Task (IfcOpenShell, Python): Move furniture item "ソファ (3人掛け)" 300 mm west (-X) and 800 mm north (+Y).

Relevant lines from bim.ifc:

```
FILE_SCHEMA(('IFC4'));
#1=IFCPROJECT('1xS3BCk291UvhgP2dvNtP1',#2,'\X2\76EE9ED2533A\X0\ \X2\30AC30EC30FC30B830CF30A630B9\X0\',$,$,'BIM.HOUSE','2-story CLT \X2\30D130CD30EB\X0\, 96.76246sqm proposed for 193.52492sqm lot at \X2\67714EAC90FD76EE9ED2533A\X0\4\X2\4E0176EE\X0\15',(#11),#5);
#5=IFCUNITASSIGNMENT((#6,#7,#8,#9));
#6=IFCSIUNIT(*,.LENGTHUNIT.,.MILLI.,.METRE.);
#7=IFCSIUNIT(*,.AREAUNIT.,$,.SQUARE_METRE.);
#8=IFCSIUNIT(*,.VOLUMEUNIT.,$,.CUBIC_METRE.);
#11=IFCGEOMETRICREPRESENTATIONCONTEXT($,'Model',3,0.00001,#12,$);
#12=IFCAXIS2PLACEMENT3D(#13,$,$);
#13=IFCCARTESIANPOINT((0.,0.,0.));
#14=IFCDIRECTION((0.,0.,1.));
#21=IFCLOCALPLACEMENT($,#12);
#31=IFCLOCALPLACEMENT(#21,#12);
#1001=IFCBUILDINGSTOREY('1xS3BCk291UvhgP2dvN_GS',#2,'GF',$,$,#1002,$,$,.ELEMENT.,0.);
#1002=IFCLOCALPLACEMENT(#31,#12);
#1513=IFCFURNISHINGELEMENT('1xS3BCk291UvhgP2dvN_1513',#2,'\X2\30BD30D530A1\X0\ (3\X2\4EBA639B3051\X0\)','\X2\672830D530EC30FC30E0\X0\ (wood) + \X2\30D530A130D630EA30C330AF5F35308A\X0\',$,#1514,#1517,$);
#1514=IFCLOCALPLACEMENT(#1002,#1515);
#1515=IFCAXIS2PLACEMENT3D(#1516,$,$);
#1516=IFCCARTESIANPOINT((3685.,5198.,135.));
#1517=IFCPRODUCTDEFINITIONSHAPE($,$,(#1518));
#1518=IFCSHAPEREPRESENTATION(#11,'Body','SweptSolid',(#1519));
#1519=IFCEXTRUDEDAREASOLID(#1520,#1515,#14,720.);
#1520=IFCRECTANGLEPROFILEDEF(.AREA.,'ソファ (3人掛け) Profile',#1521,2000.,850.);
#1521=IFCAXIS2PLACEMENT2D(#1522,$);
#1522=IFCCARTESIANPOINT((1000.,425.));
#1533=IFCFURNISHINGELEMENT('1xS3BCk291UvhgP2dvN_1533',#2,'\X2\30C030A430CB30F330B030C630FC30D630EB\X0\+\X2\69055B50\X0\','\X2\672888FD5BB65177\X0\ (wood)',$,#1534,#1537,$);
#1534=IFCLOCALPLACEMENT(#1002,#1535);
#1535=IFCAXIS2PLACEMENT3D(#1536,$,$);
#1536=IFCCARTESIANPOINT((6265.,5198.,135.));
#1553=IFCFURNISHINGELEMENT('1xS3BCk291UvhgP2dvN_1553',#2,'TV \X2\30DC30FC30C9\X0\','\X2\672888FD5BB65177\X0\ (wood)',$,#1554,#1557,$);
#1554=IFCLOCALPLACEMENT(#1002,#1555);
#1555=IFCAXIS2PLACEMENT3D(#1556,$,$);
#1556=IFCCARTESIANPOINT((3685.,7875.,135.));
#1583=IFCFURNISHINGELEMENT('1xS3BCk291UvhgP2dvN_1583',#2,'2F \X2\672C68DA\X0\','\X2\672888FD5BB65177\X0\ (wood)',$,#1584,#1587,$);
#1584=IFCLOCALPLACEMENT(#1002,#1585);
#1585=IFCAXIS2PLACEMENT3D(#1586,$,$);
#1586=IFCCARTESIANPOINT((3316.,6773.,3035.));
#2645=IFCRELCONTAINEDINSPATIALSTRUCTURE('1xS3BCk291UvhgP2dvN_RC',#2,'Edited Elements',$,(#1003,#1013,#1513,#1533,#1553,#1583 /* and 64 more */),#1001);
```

```python
import ifcopenshell
import ifcopenshell.api.geometry
import ifcopenshell.util.placement

model = ifcopenshell.open("bim.ifc")

item = model.by_guid("1xS3BCk291UvhgP2dvN_1513")
matrix = ifcopenshell.util.placement.get_local_placement(item.ObjectPlacement)
matrix[0, 3] -= 300.0
matrix[1, 3] += 800.0
ifcopenshell.api.geometry.edit_object_placement(model, product=item, matrix=matrix, is_si=False)

print(ifcopenshell.util.placement.get_local_placement(item.ObjectPlacement).round(3) + 0.0)

model.write("bim_v2.ifc")
```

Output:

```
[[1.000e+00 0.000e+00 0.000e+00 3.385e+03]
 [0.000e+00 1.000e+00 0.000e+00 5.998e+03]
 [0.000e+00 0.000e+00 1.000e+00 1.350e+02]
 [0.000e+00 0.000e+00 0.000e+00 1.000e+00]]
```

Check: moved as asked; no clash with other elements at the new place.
